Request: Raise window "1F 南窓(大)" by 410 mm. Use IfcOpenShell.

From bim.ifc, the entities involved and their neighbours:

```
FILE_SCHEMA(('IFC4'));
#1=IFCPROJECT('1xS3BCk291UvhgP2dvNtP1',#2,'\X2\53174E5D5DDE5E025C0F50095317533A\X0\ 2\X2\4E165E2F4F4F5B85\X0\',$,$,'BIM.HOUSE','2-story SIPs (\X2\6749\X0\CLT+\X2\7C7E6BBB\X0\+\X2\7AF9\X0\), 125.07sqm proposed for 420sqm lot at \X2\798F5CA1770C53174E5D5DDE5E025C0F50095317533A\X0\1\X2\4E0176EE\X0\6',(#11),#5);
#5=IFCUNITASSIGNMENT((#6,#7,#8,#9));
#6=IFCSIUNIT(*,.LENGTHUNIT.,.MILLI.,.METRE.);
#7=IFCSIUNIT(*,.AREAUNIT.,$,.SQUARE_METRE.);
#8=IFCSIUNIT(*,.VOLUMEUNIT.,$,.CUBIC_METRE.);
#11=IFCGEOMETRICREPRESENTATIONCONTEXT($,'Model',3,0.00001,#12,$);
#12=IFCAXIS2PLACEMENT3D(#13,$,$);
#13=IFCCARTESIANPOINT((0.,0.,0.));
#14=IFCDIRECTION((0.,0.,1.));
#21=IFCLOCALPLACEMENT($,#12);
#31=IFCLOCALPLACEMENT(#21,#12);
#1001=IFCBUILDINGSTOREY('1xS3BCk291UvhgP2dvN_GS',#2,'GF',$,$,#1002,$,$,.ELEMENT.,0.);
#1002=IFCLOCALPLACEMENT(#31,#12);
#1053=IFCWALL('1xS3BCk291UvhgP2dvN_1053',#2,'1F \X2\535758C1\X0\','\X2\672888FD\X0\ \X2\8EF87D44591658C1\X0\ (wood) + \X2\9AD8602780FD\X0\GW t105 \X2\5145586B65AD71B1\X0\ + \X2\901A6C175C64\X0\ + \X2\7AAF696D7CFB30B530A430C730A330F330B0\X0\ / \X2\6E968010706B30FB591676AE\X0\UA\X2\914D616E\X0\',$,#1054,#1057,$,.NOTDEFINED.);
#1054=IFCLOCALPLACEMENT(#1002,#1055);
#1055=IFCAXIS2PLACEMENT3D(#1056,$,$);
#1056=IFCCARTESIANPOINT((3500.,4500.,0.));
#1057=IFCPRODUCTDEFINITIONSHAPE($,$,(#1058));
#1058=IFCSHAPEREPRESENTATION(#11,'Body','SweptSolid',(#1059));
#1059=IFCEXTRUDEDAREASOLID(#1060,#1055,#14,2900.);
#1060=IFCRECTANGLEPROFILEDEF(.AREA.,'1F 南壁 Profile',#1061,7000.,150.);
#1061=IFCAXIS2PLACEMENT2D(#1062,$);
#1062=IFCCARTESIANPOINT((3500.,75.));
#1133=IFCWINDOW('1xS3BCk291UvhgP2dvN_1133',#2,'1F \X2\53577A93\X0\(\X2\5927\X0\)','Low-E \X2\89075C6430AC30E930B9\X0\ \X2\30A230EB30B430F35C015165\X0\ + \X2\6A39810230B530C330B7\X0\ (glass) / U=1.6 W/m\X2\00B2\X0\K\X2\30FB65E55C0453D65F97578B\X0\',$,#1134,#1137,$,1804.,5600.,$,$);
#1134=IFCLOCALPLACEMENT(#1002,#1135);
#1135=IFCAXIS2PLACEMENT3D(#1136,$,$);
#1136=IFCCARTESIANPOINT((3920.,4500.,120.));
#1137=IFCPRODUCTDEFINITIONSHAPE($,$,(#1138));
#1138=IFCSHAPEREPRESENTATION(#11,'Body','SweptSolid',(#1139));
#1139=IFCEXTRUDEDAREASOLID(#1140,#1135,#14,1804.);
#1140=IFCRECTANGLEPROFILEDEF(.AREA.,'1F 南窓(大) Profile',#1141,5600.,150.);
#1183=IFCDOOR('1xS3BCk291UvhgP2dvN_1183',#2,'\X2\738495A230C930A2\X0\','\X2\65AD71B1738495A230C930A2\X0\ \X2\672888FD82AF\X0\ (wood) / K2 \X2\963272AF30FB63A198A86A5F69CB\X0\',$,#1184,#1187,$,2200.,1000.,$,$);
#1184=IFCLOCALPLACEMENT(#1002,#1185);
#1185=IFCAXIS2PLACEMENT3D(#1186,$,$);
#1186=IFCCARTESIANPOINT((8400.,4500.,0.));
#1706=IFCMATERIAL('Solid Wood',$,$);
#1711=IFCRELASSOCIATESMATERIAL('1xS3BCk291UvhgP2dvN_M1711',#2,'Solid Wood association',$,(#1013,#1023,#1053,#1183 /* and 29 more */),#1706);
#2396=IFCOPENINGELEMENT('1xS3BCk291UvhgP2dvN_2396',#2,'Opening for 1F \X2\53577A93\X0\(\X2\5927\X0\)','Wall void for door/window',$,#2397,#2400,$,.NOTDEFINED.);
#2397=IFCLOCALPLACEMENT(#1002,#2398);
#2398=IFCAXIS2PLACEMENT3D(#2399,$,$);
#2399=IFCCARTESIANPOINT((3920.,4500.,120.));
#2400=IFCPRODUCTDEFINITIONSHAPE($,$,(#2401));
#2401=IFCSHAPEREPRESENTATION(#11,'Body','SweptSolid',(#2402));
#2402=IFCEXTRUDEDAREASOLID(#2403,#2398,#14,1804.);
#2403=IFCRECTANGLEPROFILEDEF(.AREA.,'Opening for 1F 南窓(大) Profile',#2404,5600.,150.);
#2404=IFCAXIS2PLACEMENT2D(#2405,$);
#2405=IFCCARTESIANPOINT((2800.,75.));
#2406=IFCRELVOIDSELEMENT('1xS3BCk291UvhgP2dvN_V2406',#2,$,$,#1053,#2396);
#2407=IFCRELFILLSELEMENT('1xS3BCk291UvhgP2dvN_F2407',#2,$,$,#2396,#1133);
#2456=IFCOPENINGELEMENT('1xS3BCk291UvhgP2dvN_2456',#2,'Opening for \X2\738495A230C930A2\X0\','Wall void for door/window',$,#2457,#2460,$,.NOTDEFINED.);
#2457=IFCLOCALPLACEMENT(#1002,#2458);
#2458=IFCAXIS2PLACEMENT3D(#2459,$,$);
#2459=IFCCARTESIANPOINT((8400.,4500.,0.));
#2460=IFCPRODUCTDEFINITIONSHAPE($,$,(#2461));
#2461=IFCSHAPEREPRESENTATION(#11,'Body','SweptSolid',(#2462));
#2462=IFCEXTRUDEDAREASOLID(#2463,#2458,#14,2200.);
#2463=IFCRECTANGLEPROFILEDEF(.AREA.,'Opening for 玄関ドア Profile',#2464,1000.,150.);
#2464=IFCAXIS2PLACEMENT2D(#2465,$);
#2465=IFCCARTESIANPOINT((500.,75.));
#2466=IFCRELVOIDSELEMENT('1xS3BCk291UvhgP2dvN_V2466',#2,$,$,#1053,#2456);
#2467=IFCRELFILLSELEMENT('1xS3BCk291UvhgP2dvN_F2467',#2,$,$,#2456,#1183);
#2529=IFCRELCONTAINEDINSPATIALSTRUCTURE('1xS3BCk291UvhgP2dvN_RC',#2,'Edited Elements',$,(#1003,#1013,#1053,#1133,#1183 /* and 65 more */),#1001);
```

```python
import numpy as np
import ifcopenshell
import ifcopenshell.api.geometry
import ifcopenshell.util.placement
import ifcopenshell.util.unit

model = ifcopenshell.open("bim.ifc")
unit_scale = ifcopenshell.util.unit.calculate_unit_scale(model)

window = model.by_guid("1xS3BCk291UvhgP2dvN_1133")
opening = window.FillsVoids[0].RelatingOpeningElement
dz = 0.41 / unit_scale

shift = np.array([0.0, 0.0, dz])
# The window is not placed relative to its opening, so move both.
for product in (opening, window):
    matrix = ifcopenshell.util.placement.get_local_placement(product.ObjectPlacement)
    matrix[:3, 3] += shift
    ifcopenshell.api.geometry.edit_object_placement(model, product=product, matrix=matrix, is_si=False)

print(f"moved by {dz * unit_scale:+.3f} m")

model.write("bim_rev.ifc")
```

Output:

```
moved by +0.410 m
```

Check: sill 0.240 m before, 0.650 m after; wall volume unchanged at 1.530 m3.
